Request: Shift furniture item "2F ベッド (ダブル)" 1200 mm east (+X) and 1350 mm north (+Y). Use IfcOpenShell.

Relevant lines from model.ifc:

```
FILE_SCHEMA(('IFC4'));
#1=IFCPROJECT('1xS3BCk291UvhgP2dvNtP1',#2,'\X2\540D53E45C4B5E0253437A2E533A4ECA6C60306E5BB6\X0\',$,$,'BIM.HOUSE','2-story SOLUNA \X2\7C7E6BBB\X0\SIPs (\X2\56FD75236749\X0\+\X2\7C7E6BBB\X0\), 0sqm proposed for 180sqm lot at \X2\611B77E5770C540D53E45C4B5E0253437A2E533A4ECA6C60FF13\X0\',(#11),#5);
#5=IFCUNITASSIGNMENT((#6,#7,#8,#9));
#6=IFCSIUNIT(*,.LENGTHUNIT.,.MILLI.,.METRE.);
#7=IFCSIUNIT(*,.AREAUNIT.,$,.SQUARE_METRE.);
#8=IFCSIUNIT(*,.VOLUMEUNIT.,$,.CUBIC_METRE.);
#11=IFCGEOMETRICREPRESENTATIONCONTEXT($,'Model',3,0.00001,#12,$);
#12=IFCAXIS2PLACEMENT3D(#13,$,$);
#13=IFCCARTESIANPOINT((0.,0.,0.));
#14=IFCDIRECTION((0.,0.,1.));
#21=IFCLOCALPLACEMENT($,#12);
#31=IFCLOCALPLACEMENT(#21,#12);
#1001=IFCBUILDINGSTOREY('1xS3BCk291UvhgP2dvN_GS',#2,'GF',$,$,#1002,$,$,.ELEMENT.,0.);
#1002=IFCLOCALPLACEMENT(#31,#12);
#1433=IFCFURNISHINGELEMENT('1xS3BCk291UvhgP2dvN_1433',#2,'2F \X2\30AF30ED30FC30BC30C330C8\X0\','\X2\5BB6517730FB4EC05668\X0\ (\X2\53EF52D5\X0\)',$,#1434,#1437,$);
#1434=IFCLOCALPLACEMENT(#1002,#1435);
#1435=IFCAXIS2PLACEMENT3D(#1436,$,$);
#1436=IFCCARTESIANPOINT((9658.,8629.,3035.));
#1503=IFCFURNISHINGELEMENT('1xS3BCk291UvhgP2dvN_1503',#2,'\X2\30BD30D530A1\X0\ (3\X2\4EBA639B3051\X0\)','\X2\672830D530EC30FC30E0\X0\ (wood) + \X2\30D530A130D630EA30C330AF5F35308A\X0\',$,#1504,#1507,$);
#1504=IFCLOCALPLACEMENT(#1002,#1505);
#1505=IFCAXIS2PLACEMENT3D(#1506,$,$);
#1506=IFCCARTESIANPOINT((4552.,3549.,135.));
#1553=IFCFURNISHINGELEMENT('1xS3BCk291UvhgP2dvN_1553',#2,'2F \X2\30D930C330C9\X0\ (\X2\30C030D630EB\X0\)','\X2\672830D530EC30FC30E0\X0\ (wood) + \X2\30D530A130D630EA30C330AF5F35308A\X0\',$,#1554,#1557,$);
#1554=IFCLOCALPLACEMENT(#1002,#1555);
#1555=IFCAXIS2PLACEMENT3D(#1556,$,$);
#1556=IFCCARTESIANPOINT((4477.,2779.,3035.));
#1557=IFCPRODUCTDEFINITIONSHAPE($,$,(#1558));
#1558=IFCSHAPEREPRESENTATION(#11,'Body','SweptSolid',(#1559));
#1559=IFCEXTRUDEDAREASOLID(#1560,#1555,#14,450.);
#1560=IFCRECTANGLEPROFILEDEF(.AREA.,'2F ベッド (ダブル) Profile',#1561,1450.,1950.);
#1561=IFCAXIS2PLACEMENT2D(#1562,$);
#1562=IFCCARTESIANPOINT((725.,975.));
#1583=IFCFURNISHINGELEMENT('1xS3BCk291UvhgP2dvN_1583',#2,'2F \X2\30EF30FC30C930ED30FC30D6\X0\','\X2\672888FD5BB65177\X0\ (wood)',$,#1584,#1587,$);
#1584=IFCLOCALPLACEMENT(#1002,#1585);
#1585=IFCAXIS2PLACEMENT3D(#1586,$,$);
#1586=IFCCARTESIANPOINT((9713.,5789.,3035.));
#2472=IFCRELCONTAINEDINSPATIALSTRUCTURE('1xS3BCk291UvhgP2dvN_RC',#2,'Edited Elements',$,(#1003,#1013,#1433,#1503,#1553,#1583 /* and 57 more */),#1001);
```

```python
import ifcopenshell
import ifcopenshell.api.geometry
import ifcopenshell.util.placement
import ifcopenshell.util.unit

model = ifcopenshell.open("model.ifc")
unit_scale = ifcopenshell.util.unit.calculate_unit_scale(model)

item = model.by_guid("1xS3BCk291UvhgP2dvN_1553")
matrix = ifcopenshell.util.placement.get_local_placement(item.ObjectPlacement)
matrix[0, 3] += 1.2 / unit_scale
matrix[1, 3] += 1.35 / unit_scale
ifcopenshell.api.geometry.edit_object_placement(model, product=item, matrix=matrix, is_si=False)

print(ifcopenshell.util.placement.get_local_placement(item.ObjectPlacement).round(3) + 0.0)

model.write("model-out.ifc")
```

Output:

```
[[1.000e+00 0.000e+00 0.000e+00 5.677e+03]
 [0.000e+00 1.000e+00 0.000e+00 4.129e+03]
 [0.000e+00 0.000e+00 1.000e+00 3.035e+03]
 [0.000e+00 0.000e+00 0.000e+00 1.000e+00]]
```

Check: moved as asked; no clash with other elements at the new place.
